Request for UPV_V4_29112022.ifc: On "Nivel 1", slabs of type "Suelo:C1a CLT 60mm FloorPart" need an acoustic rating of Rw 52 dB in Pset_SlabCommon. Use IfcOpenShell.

First a look at what the model holds.

```python
import ifcopenshell
import ifcopenshell.util.element

model = ifcopenshell.open("UPV_V4_29112022.ifc")
print(model.schema)
storey = next(s for s in model.by_type("IfcBuildingStorey") if s.Name == "Nivel 1")
slabs = [e for e in ifcopenshell.util.element.get_decomposition(storey) if e.is_a("IfcSlab")]
seen = {}
for e in slabs:
    element_type = ifcopenshell.util.element.get_type(e)
    key = (element_type.Name if element_type != e and element_type else None, ifcopenshell.util.element.get_pset(e, "Pset_SlabCommon", "AcousticRating"))
    seen[key] = seen.get(key, 0) + 1
for (name, value), count in sorted(seen.items(), key=str):
    print(count, "x", name, "|", value)
```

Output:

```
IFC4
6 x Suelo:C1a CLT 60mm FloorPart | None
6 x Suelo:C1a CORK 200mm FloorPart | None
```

```python
import ifcopenshell
import ifcopenshell.api.pset
import ifcopenshell.util.element

model = ifcopenshell.open("UPV_V4_29112022.ifc")

storey = next(s for s in model.by_type("IfcBuildingStorey") if s.Name == "Nivel 1")
slabs = [e for e in ifcopenshell.util.element.get_decomposition(storey) if e.is_a("IfcSlab")]

count = 0
for e in slabs:
    element_type = ifcopenshell.util.element.get_type(e)
    if element_type in (None, e) or element_type.Name != "Suelo:C1a CLT 60mm FloorPart":
        continue
    # add_pset returns the element's existing set when there is one.
    pset = ifcopenshell.api.pset.add_pset(model, product=e, name="Pset_SlabCommon")
    ifcopenshell.api.pset.edit_pset(model, pset=pset, properties={"AcousticRating": "Rw 52 dB"})
    count += 1

print(count, "slabs updated")

model.write("UPV_V4_29112022-out.ifc")
```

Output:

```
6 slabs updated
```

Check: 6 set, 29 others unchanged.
